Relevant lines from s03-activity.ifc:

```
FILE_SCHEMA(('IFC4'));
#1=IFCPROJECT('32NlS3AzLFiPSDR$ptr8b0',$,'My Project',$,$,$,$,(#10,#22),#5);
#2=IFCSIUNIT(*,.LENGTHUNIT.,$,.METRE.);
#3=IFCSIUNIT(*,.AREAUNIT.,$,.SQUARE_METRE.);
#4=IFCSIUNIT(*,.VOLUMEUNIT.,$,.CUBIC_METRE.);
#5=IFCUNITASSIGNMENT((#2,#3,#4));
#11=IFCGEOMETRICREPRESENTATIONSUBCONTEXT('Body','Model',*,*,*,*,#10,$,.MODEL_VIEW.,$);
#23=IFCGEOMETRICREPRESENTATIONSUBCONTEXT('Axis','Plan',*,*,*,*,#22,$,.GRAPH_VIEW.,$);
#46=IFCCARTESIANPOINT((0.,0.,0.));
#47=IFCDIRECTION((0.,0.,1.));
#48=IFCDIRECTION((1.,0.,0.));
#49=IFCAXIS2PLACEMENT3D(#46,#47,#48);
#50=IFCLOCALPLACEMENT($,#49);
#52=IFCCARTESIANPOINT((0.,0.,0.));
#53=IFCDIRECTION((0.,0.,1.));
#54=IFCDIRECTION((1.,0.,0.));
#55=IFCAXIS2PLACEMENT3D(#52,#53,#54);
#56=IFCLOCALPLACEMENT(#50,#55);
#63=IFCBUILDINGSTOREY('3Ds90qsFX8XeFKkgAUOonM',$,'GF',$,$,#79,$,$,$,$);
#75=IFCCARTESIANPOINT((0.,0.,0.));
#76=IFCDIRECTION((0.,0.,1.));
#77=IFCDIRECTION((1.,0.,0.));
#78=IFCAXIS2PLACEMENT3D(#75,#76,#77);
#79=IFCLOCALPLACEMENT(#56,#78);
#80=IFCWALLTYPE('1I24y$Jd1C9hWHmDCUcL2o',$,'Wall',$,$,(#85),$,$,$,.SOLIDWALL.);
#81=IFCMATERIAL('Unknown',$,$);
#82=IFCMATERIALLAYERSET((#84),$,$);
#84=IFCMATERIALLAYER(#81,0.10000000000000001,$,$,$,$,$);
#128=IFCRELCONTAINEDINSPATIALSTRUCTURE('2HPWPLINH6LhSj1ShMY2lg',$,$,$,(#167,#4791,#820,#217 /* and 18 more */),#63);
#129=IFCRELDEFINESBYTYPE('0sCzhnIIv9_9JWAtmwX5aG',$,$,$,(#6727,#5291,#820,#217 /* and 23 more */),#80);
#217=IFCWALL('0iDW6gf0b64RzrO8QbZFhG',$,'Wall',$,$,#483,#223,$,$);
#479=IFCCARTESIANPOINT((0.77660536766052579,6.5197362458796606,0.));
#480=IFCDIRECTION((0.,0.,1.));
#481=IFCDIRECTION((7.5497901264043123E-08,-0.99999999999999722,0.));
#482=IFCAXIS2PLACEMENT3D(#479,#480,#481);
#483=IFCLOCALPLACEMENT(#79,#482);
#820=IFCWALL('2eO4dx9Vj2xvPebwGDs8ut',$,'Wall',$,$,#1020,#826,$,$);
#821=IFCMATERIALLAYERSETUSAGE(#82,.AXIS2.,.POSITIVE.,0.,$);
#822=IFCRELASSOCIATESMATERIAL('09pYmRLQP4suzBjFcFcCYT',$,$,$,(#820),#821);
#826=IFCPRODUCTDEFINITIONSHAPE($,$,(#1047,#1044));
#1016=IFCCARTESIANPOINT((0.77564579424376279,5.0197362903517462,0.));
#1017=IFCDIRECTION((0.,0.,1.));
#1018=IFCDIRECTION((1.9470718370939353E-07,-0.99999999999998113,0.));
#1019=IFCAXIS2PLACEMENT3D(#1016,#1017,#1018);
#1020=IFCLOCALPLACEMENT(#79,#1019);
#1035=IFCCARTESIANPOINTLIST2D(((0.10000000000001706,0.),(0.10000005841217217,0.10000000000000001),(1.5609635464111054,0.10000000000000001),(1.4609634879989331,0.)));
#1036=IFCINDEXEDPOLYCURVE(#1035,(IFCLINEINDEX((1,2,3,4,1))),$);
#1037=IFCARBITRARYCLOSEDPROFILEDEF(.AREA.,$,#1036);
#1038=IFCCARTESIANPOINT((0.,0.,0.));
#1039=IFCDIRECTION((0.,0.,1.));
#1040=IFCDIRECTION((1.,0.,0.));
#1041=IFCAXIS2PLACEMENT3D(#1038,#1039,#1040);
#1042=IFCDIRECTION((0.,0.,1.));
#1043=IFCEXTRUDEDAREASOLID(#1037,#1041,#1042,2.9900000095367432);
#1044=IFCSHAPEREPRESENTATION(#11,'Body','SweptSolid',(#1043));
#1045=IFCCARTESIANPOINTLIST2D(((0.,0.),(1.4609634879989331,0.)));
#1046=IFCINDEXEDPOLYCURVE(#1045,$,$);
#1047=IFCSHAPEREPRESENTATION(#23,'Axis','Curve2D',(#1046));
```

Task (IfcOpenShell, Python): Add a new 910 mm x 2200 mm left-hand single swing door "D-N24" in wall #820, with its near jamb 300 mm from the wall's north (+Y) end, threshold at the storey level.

```python
import numpy as np
import ifcopenshell
import ifcopenshell.api.feature
import ifcopenshell.api.geometry
import ifcopenshell.api.root
import ifcopenshell.api.spatial
import ifcopenshell.geom
import ifcopenshell.util.element
import ifcopenshell.util.placement
import ifcopenshell.util.representation
import ifcopenshell.util.shape
import ifcopenshell.util.unit

model = ifcopenshell.open("s03-activity.ifc")
unit_scale = ifcopenshell.util.unit.calculate_unit_scale(model)
settings = ifcopenshell.geom.settings()


def volume(element):
    """Net volume in cubic metres, openings subtracted."""
    shape = ifcopenshell.geom.create_shape(settings, element)
    return ifcopenshell.util.shape.get_volume(shape.geometry)


wall = model.by_id(820)
storey = ifcopenshell.util.element.get_container(wall, ifc_class="IfcBuildingStorey")
context = ifcopenshell.util.representation.get_context(model, "Model", "Body", "MODEL_VIEW")
before = volume(wall)

width, height, from_end, sill = 0.91, 2.2, 0.3, 0.0  # metres

# The wall runs along its own X axis, and the end named is its -X end.
wall_shape = ifcopenshell.geom.create_shape(settings, wall)
x, y, z = ifcopenshell.util.shape.get_vertices(wall_shape.geometry).T
start = x.min() + from_end
face, thickness = float(y.min()), float(y.max() - y.min())
wall_matrix = ifcopenshell.util.placement.get_local_placement(wall.ObjectPlacement)
level = ifcopenshell.util.placement.get_local_placement(storey.ObjectPlacement)[2, 3]


def in_wall(x, y):
    """Placement at x, y metres in the wall's axes, at sill height."""
    matrix = wall_matrix.copy()
    matrix[:, 3] = wall_matrix @ np.array([x / unit_scale, y / unit_scale, 0.0, 1.0])
    matrix[2, 3] = level + sill / unit_scale
    return matrix


# Opening: a box that overshoots both wall faces by 50 mm.
opening = ifcopenshell.api.root.create_entity(model, ifc_class="IfcOpeningElement", predefined_type="OPENING")
box = ifcopenshell.api.geometry.add_wall_representation(
    model, context=context, length=width, height=height, thickness=thickness + 0.1
)
ifcopenshell.api.geometry.assign_representation(model, product=opening, representation=box)
ifcopenshell.api.geometry.edit_object_placement(model, product=opening, matrix=in_wall(start, face - 0.05), is_si=False)
ifcopenshell.api.feature.add_feature(model, feature=opening, element=wall)

door = ifcopenshell.api.root.create_entity(model, ifc_class="IfcDoor", name="D-N24", predefined_type="DOOR")
door.OverallWidth, door.OverallHeight = width / unit_scale, height / unit_scale
door.OperationType = "SINGLE_SWING_LEFT"
body = ifcopenshell.api.geometry.add_door_representation(
    model,
    context=context,
    overall_width=door.OverallWidth,
    overall_height=door.OverallHeight,
    operation_type="SINGLE_SWING_LEFT",
    lining_properties={"LiningDepth": thickness / unit_scale, "ThresholdDepth": thickness / unit_scale},
)
ifcopenshell.api.geometry.assign_representation(model, product=door, representation=body)
ifcopenshell.api.spatial.assign_container(model, products=[door], relating_structure=storey)
ifcopenshell.api.feature.add_filling(model, opening=opening, element=door)

# The lining spans the wall, so the door starts at the wall face.
ifcopenshell.api.geometry.edit_object_placement(model, product=door, matrix=in_wall(start, face), is_si=False)

after = volume(wall)

print(f"wall volume {before:.3f} -> {after:.3f} m3")

model.write("s03-activity-out.ifc")
```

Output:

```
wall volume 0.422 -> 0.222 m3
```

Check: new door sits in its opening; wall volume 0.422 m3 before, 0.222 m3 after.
